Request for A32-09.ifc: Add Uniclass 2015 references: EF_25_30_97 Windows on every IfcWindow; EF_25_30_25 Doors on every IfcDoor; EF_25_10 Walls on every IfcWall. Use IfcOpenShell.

First a look at what the model holds.

```python
import ifcopenshell

model = ifcopenshell.open("A32-09.ifc")
print(model.schema)
print("classifications:", [c.Name for c in model.by_type("IfcClassification")])
for ifc_class in ("IfcDoor", "IfcRoof", "IfcStair", "IfcWall", "IfcWindow"):
    print(ifc_class, len(model.by_type(ifc_class)))
```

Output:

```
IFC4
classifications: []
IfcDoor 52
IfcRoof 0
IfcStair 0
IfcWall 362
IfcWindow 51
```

```python
import ifcopenshell
import ifcopenshell.api.classification

model = ifcopenshell.open("A32-09.ifc")

system = ifcopenshell.api.classification.add_classification(model, classification="Uniclass 2015")

codes = {
    "IfcWindow": ("EF_25_30_97", "Windows"),
    "IfcDoor": ("EF_25_30_25", "Doors"),
    "IfcWall": ("EF_25_10", "Walls"),
}
for ifc_class, (code, name) in codes.items():
    products = model.by_type(ifc_class)
    ifcopenshell.api.classification.add_reference(
        model, products=products, classification=system, identification=code, name=name
    )
    print(code, len(products))

model.write("A32-09_updated.ifc")
```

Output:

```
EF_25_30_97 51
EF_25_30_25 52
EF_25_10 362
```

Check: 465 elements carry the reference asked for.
